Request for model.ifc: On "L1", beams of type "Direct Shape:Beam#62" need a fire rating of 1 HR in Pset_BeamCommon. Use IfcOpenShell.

First a look at what the model holds.

```python
import ifcopenshell
import ifcopenshell.util.element

model = ifcopenshell.open("model.ifc")
print(model.schema)
storey = next(s for s in model.by_type("IfcBuildingStorey") if s.Name == "L1")
beams = [e for e in ifcopenshell.util.element.get_decomposition(storey) if e.is_a("IfcBeam")]
seen = {}
for e in beams:
    element_type = ifcopenshell.util.element.get_type(e)
    key = (element_type.Name if element_type != e and element_type else None, ifcopenshell.util.element.get_pset(e, "Pset_BeamCommon", "FireRating"))
    seen[key] = seen.get(key, 0) + 1
for (name, value), count in sorted(seen.items(), key=str):
    print(count, "x", name, "|", value)
```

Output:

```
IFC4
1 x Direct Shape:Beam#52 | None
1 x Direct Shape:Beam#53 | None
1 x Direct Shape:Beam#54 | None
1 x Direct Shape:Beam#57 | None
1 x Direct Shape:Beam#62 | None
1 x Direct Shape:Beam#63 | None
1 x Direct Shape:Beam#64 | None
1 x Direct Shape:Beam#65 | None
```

```python
import ifcopenshell
import ifcopenshell.api.pset
import ifcopenshell.util.element

model = ifcopenshell.open("model.ifc")

storey = next(s for s in model.by_type("IfcBuildingStorey") if s.Name == "L1")
beams = [e for e in ifcopenshell.util.element.get_decomposition(storey) if e.is_a("IfcBeam")]

count = 0
for e in beams:
    element_type = ifcopenshell.util.element.get_type(e)
    if element_type in (None, e) or element_type.Name != "Direct Shape:Beam#62":
        continue
    # add_pset returns the element's existing set when there is one.
    pset = ifcopenshell.api.pset.add_pset(model, product=e, name="Pset_BeamCommon")
    ifcopenshell.api.pset.edit_pset(model, pset=pset, properties={"FireRating": "1 HR"})
    count += 1

print(count, "beams updated")

model.write("model_v2.ifc")
```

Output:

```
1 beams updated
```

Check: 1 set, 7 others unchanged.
